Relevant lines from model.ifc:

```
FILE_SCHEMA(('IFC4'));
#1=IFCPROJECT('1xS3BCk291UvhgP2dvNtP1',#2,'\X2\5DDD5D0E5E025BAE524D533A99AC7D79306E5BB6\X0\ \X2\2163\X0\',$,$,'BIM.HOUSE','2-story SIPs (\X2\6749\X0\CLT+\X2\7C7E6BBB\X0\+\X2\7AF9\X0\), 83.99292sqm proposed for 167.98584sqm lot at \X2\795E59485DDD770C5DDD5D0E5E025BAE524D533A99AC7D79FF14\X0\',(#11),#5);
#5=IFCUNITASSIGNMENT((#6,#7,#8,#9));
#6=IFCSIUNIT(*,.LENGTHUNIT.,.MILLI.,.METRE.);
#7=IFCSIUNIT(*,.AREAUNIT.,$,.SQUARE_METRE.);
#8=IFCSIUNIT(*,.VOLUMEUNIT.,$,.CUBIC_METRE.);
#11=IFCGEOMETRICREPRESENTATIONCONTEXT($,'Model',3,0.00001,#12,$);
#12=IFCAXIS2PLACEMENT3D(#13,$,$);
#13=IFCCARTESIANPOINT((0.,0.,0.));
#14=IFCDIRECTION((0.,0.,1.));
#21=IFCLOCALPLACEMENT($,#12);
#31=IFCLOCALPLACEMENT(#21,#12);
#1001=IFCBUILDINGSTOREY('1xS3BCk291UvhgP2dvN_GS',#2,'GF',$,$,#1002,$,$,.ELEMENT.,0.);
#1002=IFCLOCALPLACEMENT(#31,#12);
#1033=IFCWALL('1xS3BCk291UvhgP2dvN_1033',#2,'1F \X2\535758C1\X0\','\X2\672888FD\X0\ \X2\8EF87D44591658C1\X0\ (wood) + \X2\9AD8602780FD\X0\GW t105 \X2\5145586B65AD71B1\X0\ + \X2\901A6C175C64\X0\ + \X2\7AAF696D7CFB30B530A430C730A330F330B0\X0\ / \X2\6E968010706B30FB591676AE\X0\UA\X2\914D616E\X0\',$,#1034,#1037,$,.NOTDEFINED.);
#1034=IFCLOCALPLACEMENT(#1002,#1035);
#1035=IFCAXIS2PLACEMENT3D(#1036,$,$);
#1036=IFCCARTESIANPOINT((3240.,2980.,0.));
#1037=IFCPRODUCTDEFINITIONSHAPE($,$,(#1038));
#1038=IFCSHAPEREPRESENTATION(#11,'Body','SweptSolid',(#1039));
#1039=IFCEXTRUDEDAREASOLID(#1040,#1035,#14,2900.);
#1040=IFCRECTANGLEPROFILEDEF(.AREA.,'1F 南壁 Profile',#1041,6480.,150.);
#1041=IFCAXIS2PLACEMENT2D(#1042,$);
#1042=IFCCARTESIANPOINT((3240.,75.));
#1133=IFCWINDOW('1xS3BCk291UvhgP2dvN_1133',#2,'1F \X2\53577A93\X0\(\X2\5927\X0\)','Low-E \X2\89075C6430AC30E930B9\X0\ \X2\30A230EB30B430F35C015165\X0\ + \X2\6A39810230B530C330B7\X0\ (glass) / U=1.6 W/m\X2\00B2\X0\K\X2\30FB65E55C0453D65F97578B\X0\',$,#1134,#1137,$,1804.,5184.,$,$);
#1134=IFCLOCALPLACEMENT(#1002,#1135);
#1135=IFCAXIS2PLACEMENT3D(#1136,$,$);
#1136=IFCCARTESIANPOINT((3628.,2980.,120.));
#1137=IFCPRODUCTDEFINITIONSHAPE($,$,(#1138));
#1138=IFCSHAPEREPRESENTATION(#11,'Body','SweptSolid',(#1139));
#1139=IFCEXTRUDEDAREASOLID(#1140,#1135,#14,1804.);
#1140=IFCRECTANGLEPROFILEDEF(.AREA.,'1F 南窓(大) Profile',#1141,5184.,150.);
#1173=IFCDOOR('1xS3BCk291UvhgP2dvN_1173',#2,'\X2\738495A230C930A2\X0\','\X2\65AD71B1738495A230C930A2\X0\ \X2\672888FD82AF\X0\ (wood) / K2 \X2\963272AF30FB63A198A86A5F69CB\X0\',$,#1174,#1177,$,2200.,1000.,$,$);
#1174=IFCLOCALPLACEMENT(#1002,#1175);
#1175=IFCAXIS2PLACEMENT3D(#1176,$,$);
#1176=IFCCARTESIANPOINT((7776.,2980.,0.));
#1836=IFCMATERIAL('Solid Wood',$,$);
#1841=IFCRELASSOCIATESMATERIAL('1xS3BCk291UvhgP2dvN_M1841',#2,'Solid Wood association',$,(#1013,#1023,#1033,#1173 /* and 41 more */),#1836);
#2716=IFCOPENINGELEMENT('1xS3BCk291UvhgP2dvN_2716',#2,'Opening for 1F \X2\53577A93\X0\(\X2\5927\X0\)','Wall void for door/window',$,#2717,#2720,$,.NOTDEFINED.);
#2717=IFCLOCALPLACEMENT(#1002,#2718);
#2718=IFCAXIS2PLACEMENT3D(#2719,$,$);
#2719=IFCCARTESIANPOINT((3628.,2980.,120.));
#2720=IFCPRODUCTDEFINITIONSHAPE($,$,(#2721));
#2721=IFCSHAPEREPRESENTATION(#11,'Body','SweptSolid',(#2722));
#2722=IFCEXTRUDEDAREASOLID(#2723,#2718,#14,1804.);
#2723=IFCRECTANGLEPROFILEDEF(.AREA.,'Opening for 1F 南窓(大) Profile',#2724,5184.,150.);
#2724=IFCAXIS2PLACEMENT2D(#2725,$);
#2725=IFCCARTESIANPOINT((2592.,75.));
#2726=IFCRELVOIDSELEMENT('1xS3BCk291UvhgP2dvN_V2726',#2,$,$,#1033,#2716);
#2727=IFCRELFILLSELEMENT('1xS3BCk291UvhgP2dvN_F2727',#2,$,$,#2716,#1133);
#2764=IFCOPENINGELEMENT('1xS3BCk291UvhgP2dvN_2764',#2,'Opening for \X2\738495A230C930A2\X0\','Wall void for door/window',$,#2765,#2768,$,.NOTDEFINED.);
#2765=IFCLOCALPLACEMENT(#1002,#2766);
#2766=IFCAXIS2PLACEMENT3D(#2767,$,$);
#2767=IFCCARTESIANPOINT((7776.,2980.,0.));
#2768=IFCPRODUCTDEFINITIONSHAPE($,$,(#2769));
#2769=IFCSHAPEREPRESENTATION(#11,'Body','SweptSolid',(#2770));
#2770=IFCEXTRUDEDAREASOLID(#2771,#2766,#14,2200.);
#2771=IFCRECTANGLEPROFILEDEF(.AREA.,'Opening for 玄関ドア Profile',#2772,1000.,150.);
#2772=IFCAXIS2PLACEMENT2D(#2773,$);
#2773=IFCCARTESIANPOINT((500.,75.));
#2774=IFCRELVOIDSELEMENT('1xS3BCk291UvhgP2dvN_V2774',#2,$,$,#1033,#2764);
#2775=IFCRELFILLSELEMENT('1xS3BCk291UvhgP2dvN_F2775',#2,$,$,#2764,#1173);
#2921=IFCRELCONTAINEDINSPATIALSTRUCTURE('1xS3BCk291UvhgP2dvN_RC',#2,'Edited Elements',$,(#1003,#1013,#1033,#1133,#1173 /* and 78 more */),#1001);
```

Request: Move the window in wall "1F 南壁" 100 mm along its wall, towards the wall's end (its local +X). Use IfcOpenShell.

```python
import ifcopenshell
import ifcopenshell.api.geometry
import ifcopenshell.util.placement

model = ifcopenshell.open("model.ifc")

window = model.by_guid("1xS3BCk291UvhgP2dvN_1133")
opening = window.FillsVoids[0].RelatingOpeningElement
wall = opening.VoidsElements[0].RelatingBuildingElement

wall_matrix = ifcopenshell.util.placement.get_local_placement(wall.ObjectPlacement)
shift = wall_matrix[:3, 0] * 100.0
before = ifcopenshell.util.placement.get_local_placement(window.ObjectPlacement)[:3, 3].copy()

# The window is not placed relative to its opening, so move both.
for product in (opening, window):
    matrix = ifcopenshell.util.placement.get_local_placement(product.ObjectPlacement)
    matrix[:3, 3] += shift
    ifcopenshell.api.geometry.edit_object_placement(model, product=product, matrix=matrix, is_si=False)

after = ifcopenshell.util.placement.get_local_placement(window.ObjectPlacement)[:3, 3]
print("window moved by", (after - before).round(3) + 0.0)

model.write("model_updated.ifc")
```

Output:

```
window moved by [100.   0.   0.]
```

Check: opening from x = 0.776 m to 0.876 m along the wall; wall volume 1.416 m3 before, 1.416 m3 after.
